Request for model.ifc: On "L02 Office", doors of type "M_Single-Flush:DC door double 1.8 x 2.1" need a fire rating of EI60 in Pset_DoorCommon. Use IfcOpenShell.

First a look at what the model holds.

```python
import ifcopenshell
import ifcopenshell.util.element

model = ifcopenshell.open("model.ifc")
print(model.schema)
storey = next(s for s in model.by_type("IfcBuildingStorey") if s.Name == "L02 Office")
doors = [e for e in ifcopenshell.util.element.get_decomposition(storey) if e.is_a("IfcDoor")]
seen = {}
for e in doors:
    element_type = ifcopenshell.util.element.get_type(e)
    key = (element_type.Name if element_type != e and element_type else None, ifcopenshell.util.element.get_pset(e, "Pset_DoorCommon", "FireRating"))
    seen[key] = seen.get(key, 0) + 1
for (name, value), count in sorted(seen.items(), key=str):
    print(count, "x", name, "|", value)
```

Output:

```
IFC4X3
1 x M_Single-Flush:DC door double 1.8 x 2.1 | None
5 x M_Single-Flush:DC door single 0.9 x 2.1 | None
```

```python
import ifcopenshell
import ifcopenshell.api.pset
import ifcopenshell.util.element

model = ifcopenshell.open("model.ifc")

storey = next(s for s in model.by_type("IfcBuildingStorey") if s.Name == "L02 Office")
doors = [e for e in ifcopenshell.util.element.get_decomposition(storey) if e.is_a("IfcDoor")]

count = 0
for e in doors:
    element_type = ifcopenshell.util.element.get_type(e)
    if element_type in (None, e) or element_type.Name != "M_Single-Flush:DC door double 1.8 x 2.1":
        continue
    # add_pset returns the element's existing set when there is one.
    pset = ifcopenshell.api.pset.add_pset(model, product=e, name="Pset_DoorCommon")
    ifcopenshell.api.pset.edit_pset(model, pset=pset, properties={"FireRating": "EI60"})
    count += 1

print(count, "doors updated")

model.write("model_updated.ifc")
```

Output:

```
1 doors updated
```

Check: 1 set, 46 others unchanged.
